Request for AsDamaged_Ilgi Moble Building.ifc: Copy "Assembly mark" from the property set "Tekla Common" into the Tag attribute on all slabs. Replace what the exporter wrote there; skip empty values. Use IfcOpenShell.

First a look at what the model holds.

```python
import ifcopenshell
import ifcopenshell.util.element

model = ifcopenshell.open("AsDamaged_Ilgi Moble Building.ifc")
print(model.schema)
slabs = model.by_type("IfcSlab")
print(len(slabs), "slabs")
for e in slabs[:8]:
    source = ifcopenshell.util.element.get_pset(e, "Tekla Common", "Assembly mark")
    target = e.Tag
    print(e.id(), repr(source), repr(target), sep=" | ")
```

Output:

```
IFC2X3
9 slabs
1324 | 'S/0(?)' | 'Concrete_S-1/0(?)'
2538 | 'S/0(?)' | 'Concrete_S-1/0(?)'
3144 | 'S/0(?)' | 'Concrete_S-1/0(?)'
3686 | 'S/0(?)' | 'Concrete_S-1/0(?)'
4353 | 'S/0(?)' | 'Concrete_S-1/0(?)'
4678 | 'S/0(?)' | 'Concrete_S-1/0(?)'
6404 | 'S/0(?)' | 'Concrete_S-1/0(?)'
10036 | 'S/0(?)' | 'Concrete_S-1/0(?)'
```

```python
import ifcopenshell
import ifcopenshell.util.element

model = ifcopenshell.open("AsDamaged_Ilgi Moble Building.ifc")

count = 0
for e in model.by_type("IfcSlab"):
    value = ifcopenshell.util.element.get_pset(e, "Tekla Common", "Assembly mark")
    current = e.Tag
    if not value or not value.strip() or current == value:
        continue
    e.Tag = value
    count += 1

print(count, "slabs updated")

model.write("AsDamaged_Ilgi Moble Building_edited.ifc")
```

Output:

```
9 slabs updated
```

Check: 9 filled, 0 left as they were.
